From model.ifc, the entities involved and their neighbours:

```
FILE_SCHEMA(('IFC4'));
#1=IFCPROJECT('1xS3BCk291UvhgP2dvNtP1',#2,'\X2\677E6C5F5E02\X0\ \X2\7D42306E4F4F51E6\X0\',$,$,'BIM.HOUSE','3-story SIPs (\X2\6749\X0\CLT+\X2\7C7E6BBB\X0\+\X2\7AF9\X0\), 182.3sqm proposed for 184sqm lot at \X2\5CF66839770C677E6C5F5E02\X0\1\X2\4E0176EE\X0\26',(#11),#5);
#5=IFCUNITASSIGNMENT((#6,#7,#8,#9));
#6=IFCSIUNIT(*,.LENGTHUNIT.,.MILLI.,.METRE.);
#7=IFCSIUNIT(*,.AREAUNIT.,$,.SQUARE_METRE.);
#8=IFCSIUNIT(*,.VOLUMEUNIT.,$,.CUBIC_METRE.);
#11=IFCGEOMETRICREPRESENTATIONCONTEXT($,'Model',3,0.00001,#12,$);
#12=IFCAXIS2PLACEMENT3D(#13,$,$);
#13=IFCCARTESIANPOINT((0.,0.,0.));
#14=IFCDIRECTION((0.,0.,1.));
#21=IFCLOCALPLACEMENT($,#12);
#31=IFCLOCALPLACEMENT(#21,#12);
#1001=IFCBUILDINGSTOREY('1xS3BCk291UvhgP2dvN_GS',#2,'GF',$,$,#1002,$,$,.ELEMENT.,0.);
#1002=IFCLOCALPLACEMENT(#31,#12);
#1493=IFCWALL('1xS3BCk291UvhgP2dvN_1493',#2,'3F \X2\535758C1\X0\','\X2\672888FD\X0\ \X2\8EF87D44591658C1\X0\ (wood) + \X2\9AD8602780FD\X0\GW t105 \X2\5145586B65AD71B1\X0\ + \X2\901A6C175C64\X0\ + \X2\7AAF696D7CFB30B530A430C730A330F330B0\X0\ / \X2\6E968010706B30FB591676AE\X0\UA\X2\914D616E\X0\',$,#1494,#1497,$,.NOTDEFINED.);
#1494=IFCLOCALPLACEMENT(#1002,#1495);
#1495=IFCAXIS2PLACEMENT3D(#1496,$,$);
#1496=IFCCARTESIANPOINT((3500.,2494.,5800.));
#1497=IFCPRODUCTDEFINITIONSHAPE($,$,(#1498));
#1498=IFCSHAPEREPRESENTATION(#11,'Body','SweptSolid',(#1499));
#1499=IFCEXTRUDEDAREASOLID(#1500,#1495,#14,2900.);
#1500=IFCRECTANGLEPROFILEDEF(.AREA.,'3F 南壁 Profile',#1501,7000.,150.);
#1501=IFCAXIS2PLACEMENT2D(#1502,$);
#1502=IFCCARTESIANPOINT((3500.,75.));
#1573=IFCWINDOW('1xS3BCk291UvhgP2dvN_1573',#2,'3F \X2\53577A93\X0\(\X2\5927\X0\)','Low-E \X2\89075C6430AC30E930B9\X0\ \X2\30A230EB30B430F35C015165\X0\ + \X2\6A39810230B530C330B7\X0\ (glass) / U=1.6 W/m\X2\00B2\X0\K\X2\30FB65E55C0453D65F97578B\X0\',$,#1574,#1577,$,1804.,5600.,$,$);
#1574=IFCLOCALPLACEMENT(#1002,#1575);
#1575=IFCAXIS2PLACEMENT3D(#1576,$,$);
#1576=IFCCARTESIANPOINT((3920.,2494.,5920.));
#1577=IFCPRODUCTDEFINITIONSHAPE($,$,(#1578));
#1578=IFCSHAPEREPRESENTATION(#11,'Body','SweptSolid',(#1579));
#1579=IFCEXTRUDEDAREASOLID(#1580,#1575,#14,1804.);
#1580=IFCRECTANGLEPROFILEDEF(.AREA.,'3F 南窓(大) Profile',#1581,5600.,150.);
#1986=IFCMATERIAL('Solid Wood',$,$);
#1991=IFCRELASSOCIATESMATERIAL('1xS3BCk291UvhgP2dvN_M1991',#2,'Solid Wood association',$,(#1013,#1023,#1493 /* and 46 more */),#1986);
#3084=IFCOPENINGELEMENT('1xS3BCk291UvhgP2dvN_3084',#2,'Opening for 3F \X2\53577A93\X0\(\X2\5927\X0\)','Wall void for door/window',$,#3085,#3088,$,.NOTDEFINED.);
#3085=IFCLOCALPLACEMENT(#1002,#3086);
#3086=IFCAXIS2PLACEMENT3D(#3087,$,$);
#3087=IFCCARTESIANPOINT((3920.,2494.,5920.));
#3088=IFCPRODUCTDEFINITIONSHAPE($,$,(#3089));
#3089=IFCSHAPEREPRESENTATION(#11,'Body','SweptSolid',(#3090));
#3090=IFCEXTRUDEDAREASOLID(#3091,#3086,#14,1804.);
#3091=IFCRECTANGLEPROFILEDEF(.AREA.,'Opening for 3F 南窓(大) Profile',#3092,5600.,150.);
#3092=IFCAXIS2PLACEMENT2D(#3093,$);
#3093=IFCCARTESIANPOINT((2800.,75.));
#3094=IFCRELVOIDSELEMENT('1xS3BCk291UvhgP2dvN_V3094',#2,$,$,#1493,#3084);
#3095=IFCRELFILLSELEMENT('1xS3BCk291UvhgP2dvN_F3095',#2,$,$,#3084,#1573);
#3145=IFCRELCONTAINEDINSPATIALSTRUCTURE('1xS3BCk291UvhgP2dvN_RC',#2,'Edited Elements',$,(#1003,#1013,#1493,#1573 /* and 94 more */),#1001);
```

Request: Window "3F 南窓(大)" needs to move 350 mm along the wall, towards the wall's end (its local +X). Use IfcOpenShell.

```python
import ifcopenshell
import ifcopenshell.api.geometry
import ifcopenshell.util.placement

model = ifcopenshell.open("model.ifc")

window = model.by_guid("1xS3BCk291UvhgP2dvN_1573")
opening = window.FillsVoids[0].RelatingOpeningElement
wall = opening.VoidsElements[0].RelatingBuildingElement

wall_matrix = ifcopenshell.util.placement.get_local_placement(wall.ObjectPlacement)
shift = wall_matrix[:3, 0] * 350.0
before = ifcopenshell.util.placement.get_local_placement(window.ObjectPlacement)[:3, 3].copy()

# The window is not placed relative to its opening, so move both.
for product in (opening, window):
    matrix = ifcopenshell.util.placement.get_local_placement(product.ObjectPlacement)
    matrix[:3, 3] += shift
    ifcopenshell.api.geometry.edit_object_placement(model, product=product, matrix=matrix, is_si=False)

after = ifcopenshell.util.placement.get_local_placement(window.ObjectPlacement)[:3, 3]
print("window moved by", (after - before).round(3) + 0.0)

model.write("model_rev.ifc")
```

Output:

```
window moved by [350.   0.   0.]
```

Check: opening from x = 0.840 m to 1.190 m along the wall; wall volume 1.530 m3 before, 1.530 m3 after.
